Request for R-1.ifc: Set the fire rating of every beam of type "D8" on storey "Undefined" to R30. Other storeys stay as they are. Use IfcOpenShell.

First a look at what the model holds.

```python
import ifcopenshell
import ifcopenshell.util.element

model = ifcopenshell.open("R-1.ifc")
print(model.schema)
storey = next(s for s in model.by_type("IfcBuildingStorey") if s.Name == "Undefined")
beams = [e for e in ifcopenshell.util.element.get_decomposition(storey) if e.is_a("IfcBeam")]
seen = {}
for e in beams:
    element_type = ifcopenshell.util.element.get_type(e)
    key = (element_type.Name if element_type != e and element_type else None, ifcopenshell.util.element.get_pset(e, "Pset_BeamCommon", "FireRating"))
    seen[key] = seen.get(key, 0) + 1
for (name, value), count in sorted(seen.items(), key=str):
    print(count, "x", name, "|", value)
```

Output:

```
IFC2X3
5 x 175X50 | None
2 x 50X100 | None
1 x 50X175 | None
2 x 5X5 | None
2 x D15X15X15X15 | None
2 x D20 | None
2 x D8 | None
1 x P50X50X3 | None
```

```python
import ifcopenshell
import ifcopenshell.api.pset
import ifcopenshell.util.element

model = ifcopenshell.open("R-1.ifc")

storey = next(s for s in model.by_type("IfcBuildingStorey") if s.Name == "Undefined")
beams = [e for e in ifcopenshell.util.element.get_decomposition(storey) if e.is_a("IfcBeam")]

count = 0
for e in beams:
    element_type = ifcopenshell.util.element.get_type(e)
    if element_type in (None, e) or element_type.Name != "D8":
        continue
    found = ifcopenshell.util.element.get_pset(e, "Pset_BeamCommon", should_inherit=False)
    if found:
        pset = model.by_id(found["id"])
        if len(ifcopenshell.util.element.get_elements_by_pset(pset)) > 1:
            pset = ifcopenshell.api.pset.unshare_pset(model, products=[e], pset=pset)[0]
    else:
        pset = ifcopenshell.api.pset.add_pset(model, product=e, name="Pset_BeamCommon")
    ifcopenshell.api.pset.edit_pset(model, pset=pset, properties={"FireRating": "R30"})
    count += 1

print(count, "beams updated")

model.write("R-1_rev.ifc")
```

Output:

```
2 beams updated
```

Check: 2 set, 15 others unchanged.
